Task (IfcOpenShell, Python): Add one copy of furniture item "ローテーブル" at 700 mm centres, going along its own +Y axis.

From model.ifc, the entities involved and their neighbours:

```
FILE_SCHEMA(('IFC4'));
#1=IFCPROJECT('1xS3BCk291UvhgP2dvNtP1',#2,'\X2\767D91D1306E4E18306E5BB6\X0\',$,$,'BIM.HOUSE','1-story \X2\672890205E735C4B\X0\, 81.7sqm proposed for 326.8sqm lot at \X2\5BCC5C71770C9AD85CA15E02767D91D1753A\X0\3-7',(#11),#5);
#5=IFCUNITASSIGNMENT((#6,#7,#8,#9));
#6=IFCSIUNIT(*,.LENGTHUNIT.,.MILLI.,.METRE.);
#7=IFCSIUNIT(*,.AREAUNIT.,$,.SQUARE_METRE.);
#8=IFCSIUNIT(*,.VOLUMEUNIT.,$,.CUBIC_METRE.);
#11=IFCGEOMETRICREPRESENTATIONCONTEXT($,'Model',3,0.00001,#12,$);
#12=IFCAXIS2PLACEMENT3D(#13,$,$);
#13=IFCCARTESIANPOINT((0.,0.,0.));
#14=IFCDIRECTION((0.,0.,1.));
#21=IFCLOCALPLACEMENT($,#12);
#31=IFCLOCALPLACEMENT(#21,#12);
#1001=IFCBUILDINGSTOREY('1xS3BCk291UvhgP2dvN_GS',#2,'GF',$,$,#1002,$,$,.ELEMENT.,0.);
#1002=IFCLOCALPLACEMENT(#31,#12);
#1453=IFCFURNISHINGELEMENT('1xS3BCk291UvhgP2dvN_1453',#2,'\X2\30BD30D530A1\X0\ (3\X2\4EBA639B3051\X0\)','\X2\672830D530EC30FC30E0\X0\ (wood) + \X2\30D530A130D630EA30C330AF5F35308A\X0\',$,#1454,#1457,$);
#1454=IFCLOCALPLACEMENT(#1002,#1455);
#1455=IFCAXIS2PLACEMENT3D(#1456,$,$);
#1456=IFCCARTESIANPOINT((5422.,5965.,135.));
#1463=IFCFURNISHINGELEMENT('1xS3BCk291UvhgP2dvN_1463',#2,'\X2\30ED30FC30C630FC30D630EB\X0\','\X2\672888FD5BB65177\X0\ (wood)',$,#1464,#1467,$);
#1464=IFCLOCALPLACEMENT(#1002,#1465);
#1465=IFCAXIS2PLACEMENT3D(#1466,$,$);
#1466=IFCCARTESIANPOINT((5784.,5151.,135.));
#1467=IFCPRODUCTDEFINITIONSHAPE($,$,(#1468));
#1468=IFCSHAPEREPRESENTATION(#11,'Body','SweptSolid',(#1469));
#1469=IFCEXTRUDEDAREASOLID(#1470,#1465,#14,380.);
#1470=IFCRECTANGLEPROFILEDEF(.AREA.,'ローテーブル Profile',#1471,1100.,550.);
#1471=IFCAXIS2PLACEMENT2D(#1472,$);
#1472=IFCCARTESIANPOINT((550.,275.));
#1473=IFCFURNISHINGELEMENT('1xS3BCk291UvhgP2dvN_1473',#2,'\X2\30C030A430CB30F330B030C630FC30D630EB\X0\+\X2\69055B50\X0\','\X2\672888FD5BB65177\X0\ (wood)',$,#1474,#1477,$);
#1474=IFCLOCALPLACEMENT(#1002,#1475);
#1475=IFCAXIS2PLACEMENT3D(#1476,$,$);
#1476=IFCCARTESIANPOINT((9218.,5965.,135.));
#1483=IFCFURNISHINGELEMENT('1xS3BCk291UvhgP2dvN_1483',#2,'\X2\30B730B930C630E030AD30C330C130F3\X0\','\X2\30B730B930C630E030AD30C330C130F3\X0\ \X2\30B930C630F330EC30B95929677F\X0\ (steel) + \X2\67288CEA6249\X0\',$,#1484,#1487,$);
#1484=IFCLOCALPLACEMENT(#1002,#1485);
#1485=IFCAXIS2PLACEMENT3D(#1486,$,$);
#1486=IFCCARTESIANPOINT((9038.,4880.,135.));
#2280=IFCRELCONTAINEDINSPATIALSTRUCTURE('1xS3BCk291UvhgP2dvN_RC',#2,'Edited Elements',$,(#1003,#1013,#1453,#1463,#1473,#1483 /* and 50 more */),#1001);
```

```python
import ifcopenshell
import ifcopenshell.api.geometry
import ifcopenshell.api.root
import ifcopenshell.util.element
import ifcopenshell.util.placement

model = ifcopenshell.open("model.ifc")


def reuse_history(source, copy):
    """copy_class also copies each property set's owner history, people and application; keep the originals."""
    for rel in copy.IsDefinedBy:
        if rel.is_a("IfcRelDefinesByProperties") and (history := rel.RelatingPropertyDefinition.OwnerHistory):
            rel.RelatingPropertyDefinition.OwnerHistory = source.OwnerHistory
            ifcopenshell.util.element.remove_deep2(model, history)


source = model.by_id(1463)
base = ifcopenshell.util.placement.get_local_placement(source.ObjectPlacement)
step = base[:3, 1] * 700.0

for i in range(1, 2):
    copy = ifcopenshell.api.root.copy_class(model, product=source)
    copy.Representation = ifcopenshell.util.element.copy_deep(
        model, source.Representation, exclude=["IfcGeometricRepresentationContext", "IfcRepresentationMap"]
    )
    reuse_history(source, copy)
    matrix = base.copy()
    matrix[:3, 3] += i * step
    print("added at", matrix[:3, 3].round(3) + 0.0)
    ifcopenshell.api.geometry.edit_object_placement(model, product=copy, matrix=matrix, is_si=False)

model.write("model_edited.ifc")
```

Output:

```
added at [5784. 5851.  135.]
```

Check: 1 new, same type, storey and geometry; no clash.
